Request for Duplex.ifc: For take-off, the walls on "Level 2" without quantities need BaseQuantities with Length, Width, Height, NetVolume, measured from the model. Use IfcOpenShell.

First a look at what the model holds.

```python
import ifcopenshell
import ifcopenshell.util.element
import ifcopenshell.util.unit

model = ifcopenshell.open("Duplex.ifc")
print(model.schema)
for unit_type in ("LENGTHUNIT", "AREAUNIT", "VOLUMEUNIT"):
    print(unit_type, ifcopenshell.util.unit.calculate_unit_scale(model, unit_type))
storey = next(s for s in model.by_type("IfcBuildingStorey") if s.Name == "Level 2")
walls = [e for e in ifcopenshell.util.element.get_decomposition(storey) if e.is_a("IfcWall")]
for e in sorted(walls, key=lambda e: e.id()):
    print(e.id(), e.is_a(), e.Name, list(ifcopenshell.util.element.get_psets(e, qtos_only=True)), sep=" | ")
```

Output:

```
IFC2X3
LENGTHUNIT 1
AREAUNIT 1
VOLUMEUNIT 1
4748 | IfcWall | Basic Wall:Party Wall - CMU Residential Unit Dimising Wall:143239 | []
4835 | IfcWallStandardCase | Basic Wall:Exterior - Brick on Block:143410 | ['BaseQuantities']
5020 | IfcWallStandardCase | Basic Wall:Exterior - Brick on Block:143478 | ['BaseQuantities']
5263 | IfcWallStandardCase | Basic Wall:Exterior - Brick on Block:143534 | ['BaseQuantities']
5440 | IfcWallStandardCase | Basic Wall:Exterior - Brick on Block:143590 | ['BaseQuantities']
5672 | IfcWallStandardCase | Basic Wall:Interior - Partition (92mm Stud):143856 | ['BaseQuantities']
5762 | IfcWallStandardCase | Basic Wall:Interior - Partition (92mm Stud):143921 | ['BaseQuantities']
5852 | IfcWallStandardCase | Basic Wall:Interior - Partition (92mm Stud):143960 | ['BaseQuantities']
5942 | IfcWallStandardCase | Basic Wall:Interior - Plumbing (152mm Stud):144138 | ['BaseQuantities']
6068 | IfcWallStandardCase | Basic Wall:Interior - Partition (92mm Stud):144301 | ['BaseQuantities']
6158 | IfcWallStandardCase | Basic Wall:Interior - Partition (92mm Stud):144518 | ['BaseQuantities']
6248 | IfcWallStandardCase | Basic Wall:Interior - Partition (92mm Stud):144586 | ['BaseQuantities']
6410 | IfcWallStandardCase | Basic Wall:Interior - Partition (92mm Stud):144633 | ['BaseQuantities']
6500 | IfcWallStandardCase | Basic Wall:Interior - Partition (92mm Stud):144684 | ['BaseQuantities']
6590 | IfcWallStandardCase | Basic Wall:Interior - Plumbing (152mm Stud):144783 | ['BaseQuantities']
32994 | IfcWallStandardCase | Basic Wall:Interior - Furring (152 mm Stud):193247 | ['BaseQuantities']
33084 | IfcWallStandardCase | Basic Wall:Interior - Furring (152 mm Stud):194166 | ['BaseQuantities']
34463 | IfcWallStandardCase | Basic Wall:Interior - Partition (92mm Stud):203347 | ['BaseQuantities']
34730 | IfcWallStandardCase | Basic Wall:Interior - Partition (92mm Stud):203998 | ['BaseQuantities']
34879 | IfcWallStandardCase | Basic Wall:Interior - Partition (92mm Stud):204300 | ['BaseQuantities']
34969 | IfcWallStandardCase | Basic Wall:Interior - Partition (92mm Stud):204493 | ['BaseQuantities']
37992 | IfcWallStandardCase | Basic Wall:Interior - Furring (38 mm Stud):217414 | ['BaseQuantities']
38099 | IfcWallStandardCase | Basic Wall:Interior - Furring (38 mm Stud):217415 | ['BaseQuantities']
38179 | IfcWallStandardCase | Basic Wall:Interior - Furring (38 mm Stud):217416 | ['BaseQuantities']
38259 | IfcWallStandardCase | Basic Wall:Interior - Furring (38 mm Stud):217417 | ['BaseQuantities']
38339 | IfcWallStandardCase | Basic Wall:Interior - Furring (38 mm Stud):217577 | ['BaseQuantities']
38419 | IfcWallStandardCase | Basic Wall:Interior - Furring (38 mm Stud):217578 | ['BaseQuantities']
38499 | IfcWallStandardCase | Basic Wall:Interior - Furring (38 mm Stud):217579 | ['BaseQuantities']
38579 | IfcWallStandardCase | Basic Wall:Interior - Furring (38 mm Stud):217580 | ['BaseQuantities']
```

```python
import ifcopenshell
import ifcopenshell.api.pset
import ifcopenshell.geom
import ifcopenshell.util.element
import ifcopenshell.util.shape
import ifcopenshell.util.unit

model = ifcopenshell.open("Duplex.ifc")
unit_scale = ifcopenshell.util.unit.calculate_unit_scale(model)
volume_scale = ifcopenshell.util.unit.calculate_unit_scale(model, "VOLUMEUNIT")
settings = ifcopenshell.geom.settings()

storey = next(s for s in model.by_type("IfcBuildingStorey") if s.Name == "Level 2")
walls = [e for e in ifcopenshell.util.element.get_decomposition(storey) if e.is_a("IfcWall")]

for e in sorted(walls, key=lambda e: e.id()):
    if ifcopenshell.util.element.get_psets(e, qtos_only=True, should_inherit=False):
        continue
    # Geometry comes back in metres, in the element's own axes.
    shape = ifcopenshell.geom.create_shape(settings, e)
    values = {
        "Length": ifcopenshell.util.shape.get_x(shape.geometry) / unit_scale,
        "Width": ifcopenshell.util.shape.get_y(shape.geometry) / unit_scale,
        "Height": ifcopenshell.util.shape.get_z(shape.geometry) / unit_scale,
        "NetVolume": ifcopenshell.util.shape.get_volume(shape.geometry) / volume_scale,
    }
    qto = ifcopenshell.api.pset.add_qto(model, product=e, name="BaseQuantities")
    ifcopenshell.api.pset.edit_qto(model, qto=qto, properties=values)
    print(e.id(), {k: round(v, 3) for k, v in values.items()})

model.write("Duplex-out.ifc")
```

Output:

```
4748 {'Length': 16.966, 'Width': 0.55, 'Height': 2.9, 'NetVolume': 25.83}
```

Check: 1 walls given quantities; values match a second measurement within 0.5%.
